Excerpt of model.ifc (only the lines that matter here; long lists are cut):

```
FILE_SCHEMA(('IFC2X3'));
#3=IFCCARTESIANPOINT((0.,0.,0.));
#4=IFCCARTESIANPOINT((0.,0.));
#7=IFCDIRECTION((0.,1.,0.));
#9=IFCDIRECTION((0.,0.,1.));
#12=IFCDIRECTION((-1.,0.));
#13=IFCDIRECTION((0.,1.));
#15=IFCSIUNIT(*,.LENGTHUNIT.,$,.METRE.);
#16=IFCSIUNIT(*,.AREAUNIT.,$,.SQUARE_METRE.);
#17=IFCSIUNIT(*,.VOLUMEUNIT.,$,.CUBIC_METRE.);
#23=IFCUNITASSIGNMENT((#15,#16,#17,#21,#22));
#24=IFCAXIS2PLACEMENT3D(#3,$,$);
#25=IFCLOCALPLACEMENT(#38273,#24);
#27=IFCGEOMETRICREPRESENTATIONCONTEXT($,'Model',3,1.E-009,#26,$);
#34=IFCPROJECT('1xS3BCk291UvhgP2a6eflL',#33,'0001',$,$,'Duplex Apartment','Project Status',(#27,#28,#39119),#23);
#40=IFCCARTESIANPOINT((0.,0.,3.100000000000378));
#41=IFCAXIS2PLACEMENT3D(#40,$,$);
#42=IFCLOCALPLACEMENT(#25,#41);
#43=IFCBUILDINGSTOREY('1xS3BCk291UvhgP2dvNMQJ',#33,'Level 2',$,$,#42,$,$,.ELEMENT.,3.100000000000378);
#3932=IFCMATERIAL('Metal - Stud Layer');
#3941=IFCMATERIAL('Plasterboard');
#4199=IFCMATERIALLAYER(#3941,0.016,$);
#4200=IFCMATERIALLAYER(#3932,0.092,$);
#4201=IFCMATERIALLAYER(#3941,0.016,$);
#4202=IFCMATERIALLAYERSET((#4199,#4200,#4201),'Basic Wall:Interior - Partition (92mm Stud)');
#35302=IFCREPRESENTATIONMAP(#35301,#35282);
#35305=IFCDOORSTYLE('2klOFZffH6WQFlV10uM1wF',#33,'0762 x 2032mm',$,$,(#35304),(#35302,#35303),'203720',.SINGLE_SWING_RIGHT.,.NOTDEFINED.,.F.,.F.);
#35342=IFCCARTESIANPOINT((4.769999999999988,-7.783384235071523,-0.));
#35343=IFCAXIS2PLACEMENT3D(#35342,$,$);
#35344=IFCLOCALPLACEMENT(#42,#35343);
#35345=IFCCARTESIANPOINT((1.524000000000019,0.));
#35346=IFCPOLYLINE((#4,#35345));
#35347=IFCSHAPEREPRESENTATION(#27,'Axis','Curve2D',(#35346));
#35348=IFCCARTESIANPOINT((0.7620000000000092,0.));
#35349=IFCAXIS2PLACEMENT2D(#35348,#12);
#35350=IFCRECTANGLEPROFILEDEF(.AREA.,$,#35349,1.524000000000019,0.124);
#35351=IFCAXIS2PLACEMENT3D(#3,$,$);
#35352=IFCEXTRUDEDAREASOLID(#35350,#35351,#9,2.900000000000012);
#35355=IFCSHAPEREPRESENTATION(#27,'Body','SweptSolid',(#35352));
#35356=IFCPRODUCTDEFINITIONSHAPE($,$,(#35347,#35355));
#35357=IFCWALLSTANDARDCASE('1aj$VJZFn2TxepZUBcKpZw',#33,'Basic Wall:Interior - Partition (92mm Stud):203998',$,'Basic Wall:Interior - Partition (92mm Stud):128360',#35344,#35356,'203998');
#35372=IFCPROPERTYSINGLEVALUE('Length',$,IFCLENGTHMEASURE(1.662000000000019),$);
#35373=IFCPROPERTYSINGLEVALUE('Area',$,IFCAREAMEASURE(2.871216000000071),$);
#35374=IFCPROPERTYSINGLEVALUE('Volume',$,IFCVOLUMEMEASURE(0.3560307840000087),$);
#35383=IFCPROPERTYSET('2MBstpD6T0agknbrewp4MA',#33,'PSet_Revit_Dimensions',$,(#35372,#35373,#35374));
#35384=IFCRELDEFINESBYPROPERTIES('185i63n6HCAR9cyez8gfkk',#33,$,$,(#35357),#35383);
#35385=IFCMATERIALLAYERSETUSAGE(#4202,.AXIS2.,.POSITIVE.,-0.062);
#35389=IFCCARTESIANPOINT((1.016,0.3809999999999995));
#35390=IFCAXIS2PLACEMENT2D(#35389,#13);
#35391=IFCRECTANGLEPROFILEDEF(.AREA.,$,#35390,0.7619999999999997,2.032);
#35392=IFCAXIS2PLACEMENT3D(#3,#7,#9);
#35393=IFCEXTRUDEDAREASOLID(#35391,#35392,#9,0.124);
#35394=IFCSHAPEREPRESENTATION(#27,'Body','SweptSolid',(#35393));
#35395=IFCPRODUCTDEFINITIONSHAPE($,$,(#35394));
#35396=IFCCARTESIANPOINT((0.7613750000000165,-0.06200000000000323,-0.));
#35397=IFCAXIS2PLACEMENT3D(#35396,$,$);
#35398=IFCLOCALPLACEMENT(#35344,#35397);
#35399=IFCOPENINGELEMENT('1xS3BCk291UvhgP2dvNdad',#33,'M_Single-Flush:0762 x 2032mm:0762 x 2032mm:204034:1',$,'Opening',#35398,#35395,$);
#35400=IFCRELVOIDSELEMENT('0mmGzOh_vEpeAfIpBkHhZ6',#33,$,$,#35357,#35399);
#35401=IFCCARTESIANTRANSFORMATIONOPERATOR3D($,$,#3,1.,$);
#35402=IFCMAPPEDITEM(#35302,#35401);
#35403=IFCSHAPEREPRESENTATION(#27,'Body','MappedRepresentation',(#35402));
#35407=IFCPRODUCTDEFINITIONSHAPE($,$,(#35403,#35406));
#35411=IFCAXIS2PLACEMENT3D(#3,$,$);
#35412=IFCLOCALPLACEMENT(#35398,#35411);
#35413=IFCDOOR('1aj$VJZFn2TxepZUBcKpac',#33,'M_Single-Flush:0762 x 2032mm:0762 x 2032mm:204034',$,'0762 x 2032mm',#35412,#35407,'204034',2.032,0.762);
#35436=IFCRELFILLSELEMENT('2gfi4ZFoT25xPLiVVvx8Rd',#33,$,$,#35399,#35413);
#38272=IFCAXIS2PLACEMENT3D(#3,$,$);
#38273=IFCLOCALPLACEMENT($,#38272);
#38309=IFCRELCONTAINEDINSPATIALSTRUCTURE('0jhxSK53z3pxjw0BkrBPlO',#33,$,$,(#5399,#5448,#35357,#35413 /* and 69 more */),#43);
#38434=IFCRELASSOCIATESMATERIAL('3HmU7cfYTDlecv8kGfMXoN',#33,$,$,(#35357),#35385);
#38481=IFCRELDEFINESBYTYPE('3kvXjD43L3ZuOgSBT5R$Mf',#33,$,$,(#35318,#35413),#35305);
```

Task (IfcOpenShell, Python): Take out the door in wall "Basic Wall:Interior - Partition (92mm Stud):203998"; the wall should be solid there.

```python
import ifcopenshell
import ifcopenshell.api.feature
import ifcopenshell.api.pset
import ifcopenshell.api.root
import ifcopenshell.geom
import ifcopenshell.util.element
import ifcopenshell.util.shape
import ifcopenshell.util.unit

model = ifcopenshell.open("model.ifc")
area_scale = ifcopenshell.util.unit.calculate_unit_scale(model, "AREAUNIT")
volume_scale = ifcopenshell.util.unit.calculate_unit_scale(model, "VOLUMEUNIT")
settings = ifcopenshell.geom.settings()


def volume(element):
    """Net volume in cubic metres, openings subtracted."""
    shape = ifcopenshell.geom.create_shape(settings, element)
    return ifcopenshell.util.shape.get_volume(shape.geometry)


door = model.by_id(35413)
opening = door.FillsVoids[0].RelatingOpeningElement
wall = opening.VoidsElements[0].RelatingBuildingElement
before = volume(wall)

ifcopenshell.api.root.remove_product(model, product=door)
ifcopenshell.api.feature.remove_feature(model, feature=opening)

after = volume(wall)
thickness = 0.124  # wall thickness in metres

# Update the wall's stored quantities.
pset = model.by_id(ifcopenshell.util.element.get_pset(wall, "PSet_Revit_Dimensions", should_inherit=False)["id"])
ifcopenshell.api.pset.edit_pset(model, pset=pset, properties={
    "Area": model.create_entity("IfcAreaMeasure", after / thickness / area_scale),
    "Volume": model.create_entity("IfcVolumeMeasure", after / volume_scale),
})

print(f"wall volume {before:.3f} -> {after:.3f} m3")

model.write("model_rev.ifc")
```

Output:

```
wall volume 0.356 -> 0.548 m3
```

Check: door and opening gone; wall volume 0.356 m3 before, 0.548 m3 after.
